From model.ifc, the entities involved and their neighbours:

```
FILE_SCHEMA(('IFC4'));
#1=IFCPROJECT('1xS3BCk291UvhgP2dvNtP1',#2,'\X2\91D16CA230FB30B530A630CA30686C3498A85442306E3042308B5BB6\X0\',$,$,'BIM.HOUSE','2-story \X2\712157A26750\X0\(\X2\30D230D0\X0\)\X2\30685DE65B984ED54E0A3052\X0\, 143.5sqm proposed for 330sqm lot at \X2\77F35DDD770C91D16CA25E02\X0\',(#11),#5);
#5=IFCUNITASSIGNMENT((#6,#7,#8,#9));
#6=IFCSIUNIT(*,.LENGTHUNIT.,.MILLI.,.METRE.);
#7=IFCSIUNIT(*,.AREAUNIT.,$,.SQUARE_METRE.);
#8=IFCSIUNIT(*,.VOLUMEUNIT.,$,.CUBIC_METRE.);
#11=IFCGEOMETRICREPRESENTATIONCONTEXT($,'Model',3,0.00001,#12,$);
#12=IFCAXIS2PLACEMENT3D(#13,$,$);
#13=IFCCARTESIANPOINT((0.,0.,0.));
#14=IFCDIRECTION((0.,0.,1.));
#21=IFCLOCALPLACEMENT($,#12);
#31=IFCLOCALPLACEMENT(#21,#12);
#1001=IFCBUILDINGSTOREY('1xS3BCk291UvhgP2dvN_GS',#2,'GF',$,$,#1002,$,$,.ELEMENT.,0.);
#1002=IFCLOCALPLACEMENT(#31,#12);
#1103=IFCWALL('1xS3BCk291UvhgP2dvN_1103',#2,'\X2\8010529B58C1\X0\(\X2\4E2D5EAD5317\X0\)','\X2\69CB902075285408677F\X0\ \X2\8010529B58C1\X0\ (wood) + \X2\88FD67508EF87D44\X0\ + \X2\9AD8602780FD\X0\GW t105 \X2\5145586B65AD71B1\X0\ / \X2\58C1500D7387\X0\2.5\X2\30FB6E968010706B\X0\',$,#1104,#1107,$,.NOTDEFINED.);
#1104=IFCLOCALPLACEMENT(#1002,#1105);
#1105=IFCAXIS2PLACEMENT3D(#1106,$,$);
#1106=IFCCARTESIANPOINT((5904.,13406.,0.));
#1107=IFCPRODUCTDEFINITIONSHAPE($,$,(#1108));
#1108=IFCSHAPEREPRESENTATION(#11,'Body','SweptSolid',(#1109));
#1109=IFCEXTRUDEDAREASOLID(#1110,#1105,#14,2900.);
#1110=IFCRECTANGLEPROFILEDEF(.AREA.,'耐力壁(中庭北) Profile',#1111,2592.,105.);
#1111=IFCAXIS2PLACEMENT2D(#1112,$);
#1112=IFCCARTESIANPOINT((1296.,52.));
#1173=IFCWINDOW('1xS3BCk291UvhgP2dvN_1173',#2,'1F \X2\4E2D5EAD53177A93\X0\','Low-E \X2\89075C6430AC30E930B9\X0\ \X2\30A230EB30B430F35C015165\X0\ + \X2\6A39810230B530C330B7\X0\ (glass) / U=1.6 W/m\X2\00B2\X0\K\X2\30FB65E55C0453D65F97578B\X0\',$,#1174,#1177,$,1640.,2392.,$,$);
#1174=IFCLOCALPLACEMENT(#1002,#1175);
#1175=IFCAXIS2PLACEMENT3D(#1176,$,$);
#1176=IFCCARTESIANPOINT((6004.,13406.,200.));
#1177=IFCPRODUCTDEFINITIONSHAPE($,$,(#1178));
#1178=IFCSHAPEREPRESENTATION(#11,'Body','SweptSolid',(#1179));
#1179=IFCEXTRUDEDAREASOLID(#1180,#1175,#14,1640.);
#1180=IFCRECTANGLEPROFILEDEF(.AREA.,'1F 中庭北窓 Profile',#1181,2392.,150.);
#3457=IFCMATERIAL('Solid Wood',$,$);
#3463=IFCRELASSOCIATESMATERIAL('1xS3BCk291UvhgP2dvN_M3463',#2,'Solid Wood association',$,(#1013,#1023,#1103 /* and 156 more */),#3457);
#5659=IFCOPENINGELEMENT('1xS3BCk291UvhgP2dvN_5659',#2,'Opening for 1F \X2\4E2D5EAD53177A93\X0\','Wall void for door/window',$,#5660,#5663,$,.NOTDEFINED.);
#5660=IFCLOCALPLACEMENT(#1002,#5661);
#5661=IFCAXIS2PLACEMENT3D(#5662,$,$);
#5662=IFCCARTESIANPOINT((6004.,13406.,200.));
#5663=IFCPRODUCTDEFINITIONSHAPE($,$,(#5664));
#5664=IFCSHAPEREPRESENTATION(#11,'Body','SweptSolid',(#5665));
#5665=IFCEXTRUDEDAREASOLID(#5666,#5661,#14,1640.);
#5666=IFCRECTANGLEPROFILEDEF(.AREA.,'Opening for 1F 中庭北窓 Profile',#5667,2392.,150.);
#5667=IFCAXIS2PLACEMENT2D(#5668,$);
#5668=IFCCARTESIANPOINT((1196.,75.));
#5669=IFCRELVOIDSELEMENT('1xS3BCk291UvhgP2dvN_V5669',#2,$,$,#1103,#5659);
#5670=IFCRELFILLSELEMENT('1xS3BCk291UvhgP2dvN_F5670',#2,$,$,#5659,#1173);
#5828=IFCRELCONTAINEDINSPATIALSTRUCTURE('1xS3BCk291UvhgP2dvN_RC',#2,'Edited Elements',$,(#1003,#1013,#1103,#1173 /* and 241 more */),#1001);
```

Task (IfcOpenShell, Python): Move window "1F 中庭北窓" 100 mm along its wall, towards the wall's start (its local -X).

```python
import ifcopenshell
import ifcopenshell.api.geometry
import ifcopenshell.util.placement
import ifcopenshell.util.unit

model = ifcopenshell.open("model.ifc")
unit_scale = ifcopenshell.util.unit.calculate_unit_scale(model)

window = model.by_guid("1xS3BCk291UvhgP2dvN_1173")
opening = window.FillsVoids[0].RelatingOpeningElement
wall = opening.VoidsElements[0].RelatingBuildingElement

wall_matrix = ifcopenshell.util.placement.get_local_placement(wall.ObjectPlacement)
shift = wall_matrix[:3, 0] * -0.1 / unit_scale
before = ifcopenshell.util.placement.get_local_placement(window.ObjectPlacement)[:3, 3].copy()

# The window is not placed relative to its opening, so move both.
for product in (opening, window):
    matrix = ifcopenshell.util.placement.get_local_placement(product.ObjectPlacement)
    matrix[:3, 3] += shift
    ifcopenshell.api.geometry.edit_object_placement(model, product=product, matrix=matrix, is_si=False)

after = ifcopenshell.util.placement.get_local_placement(window.ObjectPlacement)[:3, 3]
print("window moved by", (after - before).round(3) + 0.0)

model.write("model_v2.ifc")
```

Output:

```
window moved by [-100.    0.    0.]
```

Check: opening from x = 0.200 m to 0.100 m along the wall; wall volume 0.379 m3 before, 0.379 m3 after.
